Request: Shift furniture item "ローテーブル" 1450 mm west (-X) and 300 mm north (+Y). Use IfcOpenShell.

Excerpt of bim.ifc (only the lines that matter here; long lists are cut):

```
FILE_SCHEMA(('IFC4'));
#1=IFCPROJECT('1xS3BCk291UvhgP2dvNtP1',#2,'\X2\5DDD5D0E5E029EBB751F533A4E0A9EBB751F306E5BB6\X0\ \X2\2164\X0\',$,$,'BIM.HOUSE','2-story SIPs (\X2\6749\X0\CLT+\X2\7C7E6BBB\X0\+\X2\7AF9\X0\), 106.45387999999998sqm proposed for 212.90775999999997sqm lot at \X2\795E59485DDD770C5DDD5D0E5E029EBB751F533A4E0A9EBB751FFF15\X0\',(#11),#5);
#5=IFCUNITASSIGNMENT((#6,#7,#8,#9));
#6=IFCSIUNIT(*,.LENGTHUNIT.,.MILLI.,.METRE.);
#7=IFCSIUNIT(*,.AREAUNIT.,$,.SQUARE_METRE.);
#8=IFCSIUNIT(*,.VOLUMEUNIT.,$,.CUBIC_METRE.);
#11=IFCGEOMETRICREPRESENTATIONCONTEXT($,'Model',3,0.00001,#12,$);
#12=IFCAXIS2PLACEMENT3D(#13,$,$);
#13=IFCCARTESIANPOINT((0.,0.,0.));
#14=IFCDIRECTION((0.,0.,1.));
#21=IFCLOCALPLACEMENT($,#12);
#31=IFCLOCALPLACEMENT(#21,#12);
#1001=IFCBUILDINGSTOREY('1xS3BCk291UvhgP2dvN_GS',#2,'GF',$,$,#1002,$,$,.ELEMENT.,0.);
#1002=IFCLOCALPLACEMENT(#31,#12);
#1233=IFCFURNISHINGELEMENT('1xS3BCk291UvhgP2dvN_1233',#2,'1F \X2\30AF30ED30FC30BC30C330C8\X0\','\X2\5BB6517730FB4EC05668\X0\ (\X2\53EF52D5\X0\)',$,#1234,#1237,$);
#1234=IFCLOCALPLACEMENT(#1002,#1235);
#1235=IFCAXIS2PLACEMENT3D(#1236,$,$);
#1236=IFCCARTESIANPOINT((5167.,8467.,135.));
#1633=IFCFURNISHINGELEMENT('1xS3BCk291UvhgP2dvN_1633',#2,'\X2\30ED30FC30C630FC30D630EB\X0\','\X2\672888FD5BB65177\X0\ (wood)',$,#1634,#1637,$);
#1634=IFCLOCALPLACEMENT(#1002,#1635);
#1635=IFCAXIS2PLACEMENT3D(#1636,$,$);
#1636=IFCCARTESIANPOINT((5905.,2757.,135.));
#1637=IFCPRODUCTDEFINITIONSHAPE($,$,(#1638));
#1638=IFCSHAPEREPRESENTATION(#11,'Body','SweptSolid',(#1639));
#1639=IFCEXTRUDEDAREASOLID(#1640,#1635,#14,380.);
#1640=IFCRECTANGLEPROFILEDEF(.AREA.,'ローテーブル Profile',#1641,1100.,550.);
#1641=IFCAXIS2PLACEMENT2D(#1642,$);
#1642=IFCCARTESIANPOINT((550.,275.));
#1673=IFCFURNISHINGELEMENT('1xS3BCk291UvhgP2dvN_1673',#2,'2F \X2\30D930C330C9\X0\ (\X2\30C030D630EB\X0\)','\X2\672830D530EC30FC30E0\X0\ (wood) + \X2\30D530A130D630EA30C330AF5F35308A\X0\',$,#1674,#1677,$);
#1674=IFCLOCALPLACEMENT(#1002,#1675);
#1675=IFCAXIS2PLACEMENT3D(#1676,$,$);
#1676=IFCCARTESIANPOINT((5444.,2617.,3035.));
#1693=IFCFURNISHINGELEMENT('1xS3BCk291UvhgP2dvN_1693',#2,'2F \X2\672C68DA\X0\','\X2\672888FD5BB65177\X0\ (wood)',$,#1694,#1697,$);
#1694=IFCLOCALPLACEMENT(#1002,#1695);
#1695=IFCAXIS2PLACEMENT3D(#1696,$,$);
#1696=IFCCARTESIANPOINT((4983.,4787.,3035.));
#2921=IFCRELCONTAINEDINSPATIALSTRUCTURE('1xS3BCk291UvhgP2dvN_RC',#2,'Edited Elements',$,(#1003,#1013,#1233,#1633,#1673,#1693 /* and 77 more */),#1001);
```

```python
import ifcopenshell
import ifcopenshell.api.geometry
import ifcopenshell.util.placement
import ifcopenshell.util.unit

model = ifcopenshell.open("bim.ifc")
unit_scale = ifcopenshell.util.unit.calculate_unit_scale(model)

item = model.by_id(1633)
matrix = ifcopenshell.util.placement.get_local_placement(item.ObjectPlacement)
matrix[0, 3] -= 1.45 / unit_scale
matrix[1, 3] += 0.3 / unit_scale
ifcopenshell.api.geometry.edit_object_placement(model, product=item, matrix=matrix, is_si=False)

print(ifcopenshell.util.placement.get_local_placement(item.ObjectPlacement).round(3) + 0.0)

model.write("bim_edited.ifc")
```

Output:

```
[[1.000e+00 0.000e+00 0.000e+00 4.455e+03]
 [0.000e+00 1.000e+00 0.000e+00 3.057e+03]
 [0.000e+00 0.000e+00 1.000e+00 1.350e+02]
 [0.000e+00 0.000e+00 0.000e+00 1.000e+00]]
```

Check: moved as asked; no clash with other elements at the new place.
